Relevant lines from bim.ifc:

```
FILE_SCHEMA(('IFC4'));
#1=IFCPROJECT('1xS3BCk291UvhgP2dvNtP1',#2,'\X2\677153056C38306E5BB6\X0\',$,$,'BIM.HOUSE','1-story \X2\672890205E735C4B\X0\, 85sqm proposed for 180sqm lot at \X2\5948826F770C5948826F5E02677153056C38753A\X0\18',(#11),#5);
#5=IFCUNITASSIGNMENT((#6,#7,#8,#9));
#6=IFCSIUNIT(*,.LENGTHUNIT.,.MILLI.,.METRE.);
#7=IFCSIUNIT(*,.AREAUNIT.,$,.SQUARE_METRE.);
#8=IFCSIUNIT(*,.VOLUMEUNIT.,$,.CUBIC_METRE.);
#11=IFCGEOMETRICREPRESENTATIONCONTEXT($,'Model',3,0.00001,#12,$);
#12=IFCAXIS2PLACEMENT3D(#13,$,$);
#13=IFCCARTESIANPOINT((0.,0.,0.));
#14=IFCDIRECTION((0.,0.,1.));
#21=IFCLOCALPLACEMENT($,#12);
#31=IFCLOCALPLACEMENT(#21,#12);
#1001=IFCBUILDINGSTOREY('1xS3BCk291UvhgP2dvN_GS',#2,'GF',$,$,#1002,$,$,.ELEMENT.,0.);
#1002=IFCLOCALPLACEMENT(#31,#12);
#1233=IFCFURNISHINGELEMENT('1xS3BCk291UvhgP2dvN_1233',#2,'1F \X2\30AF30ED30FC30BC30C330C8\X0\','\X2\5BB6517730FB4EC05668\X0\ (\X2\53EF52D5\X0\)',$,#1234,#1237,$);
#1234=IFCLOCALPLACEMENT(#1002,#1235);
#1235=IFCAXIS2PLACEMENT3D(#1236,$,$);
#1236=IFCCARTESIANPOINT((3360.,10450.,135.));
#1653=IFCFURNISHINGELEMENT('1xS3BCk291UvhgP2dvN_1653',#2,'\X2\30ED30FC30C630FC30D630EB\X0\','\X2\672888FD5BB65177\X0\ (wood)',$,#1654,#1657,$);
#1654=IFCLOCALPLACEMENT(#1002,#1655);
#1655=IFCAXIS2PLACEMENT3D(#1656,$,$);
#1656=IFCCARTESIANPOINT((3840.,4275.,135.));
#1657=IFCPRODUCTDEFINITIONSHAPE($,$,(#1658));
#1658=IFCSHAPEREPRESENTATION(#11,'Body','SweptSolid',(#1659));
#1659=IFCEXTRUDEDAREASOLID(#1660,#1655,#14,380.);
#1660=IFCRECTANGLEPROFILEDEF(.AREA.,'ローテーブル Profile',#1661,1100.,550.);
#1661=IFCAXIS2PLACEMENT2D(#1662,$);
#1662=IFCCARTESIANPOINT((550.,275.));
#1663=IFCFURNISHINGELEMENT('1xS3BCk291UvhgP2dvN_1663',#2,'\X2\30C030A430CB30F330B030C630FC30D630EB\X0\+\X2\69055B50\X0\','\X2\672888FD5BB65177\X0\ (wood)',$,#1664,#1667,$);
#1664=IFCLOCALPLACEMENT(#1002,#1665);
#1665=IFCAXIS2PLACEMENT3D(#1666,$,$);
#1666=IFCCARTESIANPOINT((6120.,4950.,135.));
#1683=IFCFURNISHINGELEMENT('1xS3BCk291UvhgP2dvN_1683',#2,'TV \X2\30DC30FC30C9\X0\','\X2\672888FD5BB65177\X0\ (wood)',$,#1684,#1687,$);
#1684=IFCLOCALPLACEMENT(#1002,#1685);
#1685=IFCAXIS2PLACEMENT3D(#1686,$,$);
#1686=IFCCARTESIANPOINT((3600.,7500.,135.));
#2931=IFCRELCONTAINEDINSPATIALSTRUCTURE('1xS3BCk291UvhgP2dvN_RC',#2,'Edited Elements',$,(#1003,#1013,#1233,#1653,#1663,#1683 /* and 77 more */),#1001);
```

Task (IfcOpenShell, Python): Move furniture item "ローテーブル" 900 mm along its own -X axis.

```python
import ifcopenshell
import ifcopenshell.api.geometry
import ifcopenshell.util.placement
import ifcopenshell.util.unit

model = ifcopenshell.open("bim.ifc")
unit_scale = ifcopenshell.util.unit.calculate_unit_scale(model)

item = model.by_id(1653)
matrix = ifcopenshell.util.placement.get_local_placement(item.ObjectPlacement)
matrix[:3, 3] -= matrix[:3, 0] * 0.9 / unit_scale
ifcopenshell.api.geometry.edit_object_placement(model, product=item, matrix=matrix, is_si=False)

print(ifcopenshell.util.placement.get_local_placement(item.ObjectPlacement).round(3) + 0.0)

model.write("bim_edited.ifc")
```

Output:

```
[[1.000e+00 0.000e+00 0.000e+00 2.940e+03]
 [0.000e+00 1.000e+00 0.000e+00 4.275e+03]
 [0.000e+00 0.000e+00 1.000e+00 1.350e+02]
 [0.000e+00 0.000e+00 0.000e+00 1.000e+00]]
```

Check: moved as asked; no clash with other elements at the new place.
